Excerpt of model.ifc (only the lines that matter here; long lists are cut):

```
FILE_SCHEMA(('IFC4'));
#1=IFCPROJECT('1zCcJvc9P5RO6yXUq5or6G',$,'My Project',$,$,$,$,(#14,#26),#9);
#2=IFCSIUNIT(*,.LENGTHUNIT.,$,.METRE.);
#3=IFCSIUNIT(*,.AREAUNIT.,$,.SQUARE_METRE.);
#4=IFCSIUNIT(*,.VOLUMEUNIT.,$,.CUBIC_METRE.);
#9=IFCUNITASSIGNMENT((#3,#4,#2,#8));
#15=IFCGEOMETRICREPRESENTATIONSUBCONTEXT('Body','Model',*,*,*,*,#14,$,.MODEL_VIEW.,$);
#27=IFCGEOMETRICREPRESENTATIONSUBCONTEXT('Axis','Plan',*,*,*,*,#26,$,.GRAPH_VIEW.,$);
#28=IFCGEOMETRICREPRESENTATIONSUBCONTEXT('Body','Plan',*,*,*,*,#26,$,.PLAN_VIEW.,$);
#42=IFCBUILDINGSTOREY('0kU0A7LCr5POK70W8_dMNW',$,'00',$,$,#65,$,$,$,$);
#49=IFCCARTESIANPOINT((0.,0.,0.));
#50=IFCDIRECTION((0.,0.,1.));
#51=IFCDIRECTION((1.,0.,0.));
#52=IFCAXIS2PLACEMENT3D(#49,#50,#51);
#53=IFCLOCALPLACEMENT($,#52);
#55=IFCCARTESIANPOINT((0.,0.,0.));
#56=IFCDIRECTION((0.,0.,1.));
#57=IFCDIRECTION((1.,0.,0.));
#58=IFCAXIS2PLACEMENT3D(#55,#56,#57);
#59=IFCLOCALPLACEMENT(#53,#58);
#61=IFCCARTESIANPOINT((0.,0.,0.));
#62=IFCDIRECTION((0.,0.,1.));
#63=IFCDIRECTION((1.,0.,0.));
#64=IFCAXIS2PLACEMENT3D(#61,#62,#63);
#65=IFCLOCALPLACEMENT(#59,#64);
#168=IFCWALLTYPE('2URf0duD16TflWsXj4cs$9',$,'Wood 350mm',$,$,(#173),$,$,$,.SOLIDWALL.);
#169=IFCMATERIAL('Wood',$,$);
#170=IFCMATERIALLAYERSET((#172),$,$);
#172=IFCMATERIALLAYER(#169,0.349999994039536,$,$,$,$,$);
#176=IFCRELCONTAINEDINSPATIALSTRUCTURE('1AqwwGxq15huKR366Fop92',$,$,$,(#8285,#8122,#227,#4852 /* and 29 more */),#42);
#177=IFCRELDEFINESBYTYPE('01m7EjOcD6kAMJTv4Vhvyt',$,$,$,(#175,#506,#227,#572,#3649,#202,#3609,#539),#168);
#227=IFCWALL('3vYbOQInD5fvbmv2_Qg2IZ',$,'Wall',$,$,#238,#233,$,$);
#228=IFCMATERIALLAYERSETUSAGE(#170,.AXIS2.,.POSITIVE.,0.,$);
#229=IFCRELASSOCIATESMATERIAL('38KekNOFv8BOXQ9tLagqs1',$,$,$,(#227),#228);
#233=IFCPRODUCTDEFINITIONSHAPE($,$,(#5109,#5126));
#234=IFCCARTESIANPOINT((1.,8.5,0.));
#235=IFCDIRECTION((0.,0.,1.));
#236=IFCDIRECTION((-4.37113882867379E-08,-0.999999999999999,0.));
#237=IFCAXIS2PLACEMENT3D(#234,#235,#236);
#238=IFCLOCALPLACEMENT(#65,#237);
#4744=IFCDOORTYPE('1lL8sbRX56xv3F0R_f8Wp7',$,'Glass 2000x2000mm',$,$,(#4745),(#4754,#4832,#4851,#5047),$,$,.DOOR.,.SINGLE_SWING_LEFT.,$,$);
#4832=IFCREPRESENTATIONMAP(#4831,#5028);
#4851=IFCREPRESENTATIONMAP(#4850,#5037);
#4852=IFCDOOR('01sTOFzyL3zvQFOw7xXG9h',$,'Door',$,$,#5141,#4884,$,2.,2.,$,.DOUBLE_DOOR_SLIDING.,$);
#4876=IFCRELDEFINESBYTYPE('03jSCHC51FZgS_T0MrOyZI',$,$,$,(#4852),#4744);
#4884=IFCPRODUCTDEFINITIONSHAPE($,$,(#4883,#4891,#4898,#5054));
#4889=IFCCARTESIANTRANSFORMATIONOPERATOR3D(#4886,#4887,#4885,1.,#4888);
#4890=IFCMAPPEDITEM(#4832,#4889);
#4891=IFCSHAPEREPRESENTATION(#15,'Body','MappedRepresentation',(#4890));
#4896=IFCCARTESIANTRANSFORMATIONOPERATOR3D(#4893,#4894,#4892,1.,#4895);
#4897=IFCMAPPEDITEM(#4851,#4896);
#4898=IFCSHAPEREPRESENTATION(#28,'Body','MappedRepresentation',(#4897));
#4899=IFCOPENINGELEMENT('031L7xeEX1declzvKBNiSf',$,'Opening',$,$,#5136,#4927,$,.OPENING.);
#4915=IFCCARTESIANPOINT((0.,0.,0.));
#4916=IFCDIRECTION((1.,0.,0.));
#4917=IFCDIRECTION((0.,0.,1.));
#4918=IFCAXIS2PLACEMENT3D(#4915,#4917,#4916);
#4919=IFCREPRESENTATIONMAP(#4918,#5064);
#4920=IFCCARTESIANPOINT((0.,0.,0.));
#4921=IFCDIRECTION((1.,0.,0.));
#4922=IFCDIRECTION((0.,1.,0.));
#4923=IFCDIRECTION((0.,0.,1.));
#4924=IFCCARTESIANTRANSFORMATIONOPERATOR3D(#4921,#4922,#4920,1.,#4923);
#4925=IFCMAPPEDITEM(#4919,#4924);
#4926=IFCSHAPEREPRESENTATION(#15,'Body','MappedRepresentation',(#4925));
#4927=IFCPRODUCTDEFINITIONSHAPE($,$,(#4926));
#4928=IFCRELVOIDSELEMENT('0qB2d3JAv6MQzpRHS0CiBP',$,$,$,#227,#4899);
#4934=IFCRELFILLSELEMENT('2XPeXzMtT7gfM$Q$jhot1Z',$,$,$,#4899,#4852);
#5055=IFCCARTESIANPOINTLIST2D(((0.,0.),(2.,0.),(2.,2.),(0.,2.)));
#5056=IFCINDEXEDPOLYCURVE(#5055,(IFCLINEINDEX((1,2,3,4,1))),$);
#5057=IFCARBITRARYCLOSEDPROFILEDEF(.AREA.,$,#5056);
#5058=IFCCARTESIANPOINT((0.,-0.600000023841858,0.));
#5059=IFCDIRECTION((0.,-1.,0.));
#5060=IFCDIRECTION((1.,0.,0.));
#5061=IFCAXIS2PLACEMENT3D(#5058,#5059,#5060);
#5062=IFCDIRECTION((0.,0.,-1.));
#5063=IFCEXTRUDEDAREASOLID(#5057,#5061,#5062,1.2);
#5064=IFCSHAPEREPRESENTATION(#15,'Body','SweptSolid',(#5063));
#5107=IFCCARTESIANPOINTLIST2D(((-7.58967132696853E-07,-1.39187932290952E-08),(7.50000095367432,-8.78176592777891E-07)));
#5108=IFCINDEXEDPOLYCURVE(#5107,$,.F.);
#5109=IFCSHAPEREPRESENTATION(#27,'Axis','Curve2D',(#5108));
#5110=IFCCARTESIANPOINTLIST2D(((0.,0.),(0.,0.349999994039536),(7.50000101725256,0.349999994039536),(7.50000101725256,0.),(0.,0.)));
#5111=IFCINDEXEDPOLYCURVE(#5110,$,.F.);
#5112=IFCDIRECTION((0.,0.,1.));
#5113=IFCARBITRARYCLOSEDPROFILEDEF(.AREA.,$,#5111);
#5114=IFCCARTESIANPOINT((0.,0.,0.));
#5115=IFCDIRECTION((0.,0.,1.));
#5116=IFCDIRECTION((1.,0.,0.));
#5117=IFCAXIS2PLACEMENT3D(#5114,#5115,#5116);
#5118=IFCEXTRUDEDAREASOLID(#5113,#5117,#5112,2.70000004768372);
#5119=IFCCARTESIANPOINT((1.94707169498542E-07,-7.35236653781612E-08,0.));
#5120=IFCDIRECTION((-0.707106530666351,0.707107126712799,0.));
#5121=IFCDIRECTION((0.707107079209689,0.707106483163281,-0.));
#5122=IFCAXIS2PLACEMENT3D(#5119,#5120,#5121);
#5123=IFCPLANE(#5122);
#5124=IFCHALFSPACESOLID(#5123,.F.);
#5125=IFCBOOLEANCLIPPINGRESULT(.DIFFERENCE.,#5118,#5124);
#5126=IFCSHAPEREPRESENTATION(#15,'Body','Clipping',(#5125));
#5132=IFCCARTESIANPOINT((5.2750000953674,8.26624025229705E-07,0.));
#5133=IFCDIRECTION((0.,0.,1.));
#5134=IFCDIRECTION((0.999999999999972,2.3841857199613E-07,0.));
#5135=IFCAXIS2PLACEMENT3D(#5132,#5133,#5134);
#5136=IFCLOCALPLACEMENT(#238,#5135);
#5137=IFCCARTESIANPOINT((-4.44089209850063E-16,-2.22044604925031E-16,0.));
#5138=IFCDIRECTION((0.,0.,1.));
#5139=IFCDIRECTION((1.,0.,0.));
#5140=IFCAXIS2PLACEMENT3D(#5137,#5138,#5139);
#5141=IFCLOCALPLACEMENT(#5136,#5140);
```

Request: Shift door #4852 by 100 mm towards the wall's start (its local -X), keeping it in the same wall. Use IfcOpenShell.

```python
import ifcopenshell
import ifcopenshell.api.geometry
import ifcopenshell.util.placement
import ifcopenshell.util.unit

model = ifcopenshell.open("model.ifc")
unit_scale = ifcopenshell.util.unit.calculate_unit_scale(model)

door = model.by_guid("01sTOFzyL3zvQFOw7xXG9h")
opening = door.FillsVoids[0].RelatingOpeningElement
wall = opening.VoidsElements[0].RelatingBuildingElement

wall_matrix = ifcopenshell.util.placement.get_local_placement(wall.ObjectPlacement)
shift = wall_matrix[:3, 0] * -0.1 / unit_scale
before = ifcopenshell.util.placement.get_local_placement(door.ObjectPlacement)[:3, 3].copy()

# The door is placed relative to its opening, so it follows when the opening moves.
matrix = ifcopenshell.util.placement.get_local_placement(opening.ObjectPlacement)
matrix[:3, 3] += shift
ifcopenshell.api.geometry.edit_object_placement(
    model, product=opening, matrix=matrix, is_si=False, should_transform_children=True
)

after = ifcopenshell.util.placement.get_local_placement(door.ObjectPlacement)[:3, 3]
print("door moved by", (after - before).round(3) + 0.0)

model.write("model_rev.ifc")
```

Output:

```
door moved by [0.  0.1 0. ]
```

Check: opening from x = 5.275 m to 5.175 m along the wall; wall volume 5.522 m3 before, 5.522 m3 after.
